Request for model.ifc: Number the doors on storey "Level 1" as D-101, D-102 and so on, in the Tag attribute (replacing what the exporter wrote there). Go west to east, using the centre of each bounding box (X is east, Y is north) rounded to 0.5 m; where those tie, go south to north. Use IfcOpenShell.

First a look at what the model holds.

```python
import ifcopenshell
import ifcopenshell.util.element
import ifcopenshell.util.placement

model = ifcopenshell.open("model.ifc")
print(model.schema)
storey = next(s for s in model.by_type("IfcBuildingStorey") if s.Name == "Level 1")
doors = [e for e in ifcopenshell.util.element.get_decomposition(storey) if e.is_a("IfcDoor")]
for e in sorted(doors, key=lambda e: e.id()):
    origin = ifcopenshell.util.placement.get_local_placement(e.ObjectPlacement)[:3, 3]
    print(e.id(), e.Tag, e.Name, origin.round(2) + 0.0, sep=" | ")
```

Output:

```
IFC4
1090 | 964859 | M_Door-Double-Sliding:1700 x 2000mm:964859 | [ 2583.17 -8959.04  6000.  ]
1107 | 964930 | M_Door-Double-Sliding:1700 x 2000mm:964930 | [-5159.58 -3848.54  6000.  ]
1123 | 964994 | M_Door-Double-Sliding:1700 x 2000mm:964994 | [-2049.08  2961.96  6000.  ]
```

```python
import ifcopenshell
import ifcopenshell.geom
import ifcopenshell.util.element
import ifcopenshell.util.shape

model = ifcopenshell.open("model.ifc")
settings = ifcopenshell.geom.settings()
settings.set("use-world-coords", True)


def centre(element):
    shape = ifcopenshell.geom.create_shape(settings, element)
    return ifcopenshell.util.shape.get_bbox_centroid(shape.geometry)


storey = next(s for s in model.by_type("IfcBuildingStorey") if s.Name == "Level 1")
doors = [e for e in ifcopenshell.util.element.get_decomposition(storey) if e.is_a("IfcDoor")]

# Insertion points can sit at a corner or the storey origin, so sort by the geometry (in metres).
centres = {e: centre(e) for e in doors}
doors.sort(key=lambda e: (round(centres[e][0] / 0.5), centres[e][1]))

for i, e in enumerate(doors, start=1):
    number = f"D-1{i:02d}"
    e.Tag = number
    print(e.id(), number)

model.write("model_rev.ifc")
```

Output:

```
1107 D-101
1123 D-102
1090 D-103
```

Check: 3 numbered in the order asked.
